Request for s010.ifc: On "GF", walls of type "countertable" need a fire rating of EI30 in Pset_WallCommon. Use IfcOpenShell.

First a look at what the model holds.

```python
import ifcopenshell
import ifcopenshell.util.element

model = ifcopenshell.open("s010.ifc")
print(model.schema)
storey = next(s for s in model.by_type("IfcBuildingStorey") if s.Name == "GF")
walls = [e for e in ifcopenshell.util.element.get_decomposition(storey) if e.is_a("IfcWall")]
seen = {}
for e in walls:
    element_type = ifcopenshell.util.element.get_type(e)
    key = (element_type.Name if element_type != e and element_type else None, ifcopenshell.util.element.get_pset(e, "Pset_WallCommon", "FireRating"))
    seen[key] = seen.get(key, 0) + 1
for (name, value), count in sorted(seen.items(), key=str):
    print(count, "x", name, "|", value)
```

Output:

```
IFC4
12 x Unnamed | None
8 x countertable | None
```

```python
import ifcopenshell
import ifcopenshell.api.pset
import ifcopenshell.util.element

model = ifcopenshell.open("s010.ifc")

storey = next(s for s in model.by_type("IfcBuildingStorey") if s.Name == "GF")
walls = [e for e in ifcopenshell.util.element.get_decomposition(storey) if e.is_a("IfcWall")]

count = 0
for e in walls:
    element_type = ifcopenshell.util.element.get_type(e)
    if element_type in (None, e) or element_type.Name != "countertable":
        continue
    # add_pset returns the element's existing set when there is one.
    pset = ifcopenshell.api.pset.add_pset(model, product=e, name="Pset_WallCommon")
    ifcopenshell.api.pset.edit_pset(model, pset=pset, properties={"FireRating": "EI30"})
    count += 1

print(count, "walls updated")

model.write("s010_rev.ifc")
```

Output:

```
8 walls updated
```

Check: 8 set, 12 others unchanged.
